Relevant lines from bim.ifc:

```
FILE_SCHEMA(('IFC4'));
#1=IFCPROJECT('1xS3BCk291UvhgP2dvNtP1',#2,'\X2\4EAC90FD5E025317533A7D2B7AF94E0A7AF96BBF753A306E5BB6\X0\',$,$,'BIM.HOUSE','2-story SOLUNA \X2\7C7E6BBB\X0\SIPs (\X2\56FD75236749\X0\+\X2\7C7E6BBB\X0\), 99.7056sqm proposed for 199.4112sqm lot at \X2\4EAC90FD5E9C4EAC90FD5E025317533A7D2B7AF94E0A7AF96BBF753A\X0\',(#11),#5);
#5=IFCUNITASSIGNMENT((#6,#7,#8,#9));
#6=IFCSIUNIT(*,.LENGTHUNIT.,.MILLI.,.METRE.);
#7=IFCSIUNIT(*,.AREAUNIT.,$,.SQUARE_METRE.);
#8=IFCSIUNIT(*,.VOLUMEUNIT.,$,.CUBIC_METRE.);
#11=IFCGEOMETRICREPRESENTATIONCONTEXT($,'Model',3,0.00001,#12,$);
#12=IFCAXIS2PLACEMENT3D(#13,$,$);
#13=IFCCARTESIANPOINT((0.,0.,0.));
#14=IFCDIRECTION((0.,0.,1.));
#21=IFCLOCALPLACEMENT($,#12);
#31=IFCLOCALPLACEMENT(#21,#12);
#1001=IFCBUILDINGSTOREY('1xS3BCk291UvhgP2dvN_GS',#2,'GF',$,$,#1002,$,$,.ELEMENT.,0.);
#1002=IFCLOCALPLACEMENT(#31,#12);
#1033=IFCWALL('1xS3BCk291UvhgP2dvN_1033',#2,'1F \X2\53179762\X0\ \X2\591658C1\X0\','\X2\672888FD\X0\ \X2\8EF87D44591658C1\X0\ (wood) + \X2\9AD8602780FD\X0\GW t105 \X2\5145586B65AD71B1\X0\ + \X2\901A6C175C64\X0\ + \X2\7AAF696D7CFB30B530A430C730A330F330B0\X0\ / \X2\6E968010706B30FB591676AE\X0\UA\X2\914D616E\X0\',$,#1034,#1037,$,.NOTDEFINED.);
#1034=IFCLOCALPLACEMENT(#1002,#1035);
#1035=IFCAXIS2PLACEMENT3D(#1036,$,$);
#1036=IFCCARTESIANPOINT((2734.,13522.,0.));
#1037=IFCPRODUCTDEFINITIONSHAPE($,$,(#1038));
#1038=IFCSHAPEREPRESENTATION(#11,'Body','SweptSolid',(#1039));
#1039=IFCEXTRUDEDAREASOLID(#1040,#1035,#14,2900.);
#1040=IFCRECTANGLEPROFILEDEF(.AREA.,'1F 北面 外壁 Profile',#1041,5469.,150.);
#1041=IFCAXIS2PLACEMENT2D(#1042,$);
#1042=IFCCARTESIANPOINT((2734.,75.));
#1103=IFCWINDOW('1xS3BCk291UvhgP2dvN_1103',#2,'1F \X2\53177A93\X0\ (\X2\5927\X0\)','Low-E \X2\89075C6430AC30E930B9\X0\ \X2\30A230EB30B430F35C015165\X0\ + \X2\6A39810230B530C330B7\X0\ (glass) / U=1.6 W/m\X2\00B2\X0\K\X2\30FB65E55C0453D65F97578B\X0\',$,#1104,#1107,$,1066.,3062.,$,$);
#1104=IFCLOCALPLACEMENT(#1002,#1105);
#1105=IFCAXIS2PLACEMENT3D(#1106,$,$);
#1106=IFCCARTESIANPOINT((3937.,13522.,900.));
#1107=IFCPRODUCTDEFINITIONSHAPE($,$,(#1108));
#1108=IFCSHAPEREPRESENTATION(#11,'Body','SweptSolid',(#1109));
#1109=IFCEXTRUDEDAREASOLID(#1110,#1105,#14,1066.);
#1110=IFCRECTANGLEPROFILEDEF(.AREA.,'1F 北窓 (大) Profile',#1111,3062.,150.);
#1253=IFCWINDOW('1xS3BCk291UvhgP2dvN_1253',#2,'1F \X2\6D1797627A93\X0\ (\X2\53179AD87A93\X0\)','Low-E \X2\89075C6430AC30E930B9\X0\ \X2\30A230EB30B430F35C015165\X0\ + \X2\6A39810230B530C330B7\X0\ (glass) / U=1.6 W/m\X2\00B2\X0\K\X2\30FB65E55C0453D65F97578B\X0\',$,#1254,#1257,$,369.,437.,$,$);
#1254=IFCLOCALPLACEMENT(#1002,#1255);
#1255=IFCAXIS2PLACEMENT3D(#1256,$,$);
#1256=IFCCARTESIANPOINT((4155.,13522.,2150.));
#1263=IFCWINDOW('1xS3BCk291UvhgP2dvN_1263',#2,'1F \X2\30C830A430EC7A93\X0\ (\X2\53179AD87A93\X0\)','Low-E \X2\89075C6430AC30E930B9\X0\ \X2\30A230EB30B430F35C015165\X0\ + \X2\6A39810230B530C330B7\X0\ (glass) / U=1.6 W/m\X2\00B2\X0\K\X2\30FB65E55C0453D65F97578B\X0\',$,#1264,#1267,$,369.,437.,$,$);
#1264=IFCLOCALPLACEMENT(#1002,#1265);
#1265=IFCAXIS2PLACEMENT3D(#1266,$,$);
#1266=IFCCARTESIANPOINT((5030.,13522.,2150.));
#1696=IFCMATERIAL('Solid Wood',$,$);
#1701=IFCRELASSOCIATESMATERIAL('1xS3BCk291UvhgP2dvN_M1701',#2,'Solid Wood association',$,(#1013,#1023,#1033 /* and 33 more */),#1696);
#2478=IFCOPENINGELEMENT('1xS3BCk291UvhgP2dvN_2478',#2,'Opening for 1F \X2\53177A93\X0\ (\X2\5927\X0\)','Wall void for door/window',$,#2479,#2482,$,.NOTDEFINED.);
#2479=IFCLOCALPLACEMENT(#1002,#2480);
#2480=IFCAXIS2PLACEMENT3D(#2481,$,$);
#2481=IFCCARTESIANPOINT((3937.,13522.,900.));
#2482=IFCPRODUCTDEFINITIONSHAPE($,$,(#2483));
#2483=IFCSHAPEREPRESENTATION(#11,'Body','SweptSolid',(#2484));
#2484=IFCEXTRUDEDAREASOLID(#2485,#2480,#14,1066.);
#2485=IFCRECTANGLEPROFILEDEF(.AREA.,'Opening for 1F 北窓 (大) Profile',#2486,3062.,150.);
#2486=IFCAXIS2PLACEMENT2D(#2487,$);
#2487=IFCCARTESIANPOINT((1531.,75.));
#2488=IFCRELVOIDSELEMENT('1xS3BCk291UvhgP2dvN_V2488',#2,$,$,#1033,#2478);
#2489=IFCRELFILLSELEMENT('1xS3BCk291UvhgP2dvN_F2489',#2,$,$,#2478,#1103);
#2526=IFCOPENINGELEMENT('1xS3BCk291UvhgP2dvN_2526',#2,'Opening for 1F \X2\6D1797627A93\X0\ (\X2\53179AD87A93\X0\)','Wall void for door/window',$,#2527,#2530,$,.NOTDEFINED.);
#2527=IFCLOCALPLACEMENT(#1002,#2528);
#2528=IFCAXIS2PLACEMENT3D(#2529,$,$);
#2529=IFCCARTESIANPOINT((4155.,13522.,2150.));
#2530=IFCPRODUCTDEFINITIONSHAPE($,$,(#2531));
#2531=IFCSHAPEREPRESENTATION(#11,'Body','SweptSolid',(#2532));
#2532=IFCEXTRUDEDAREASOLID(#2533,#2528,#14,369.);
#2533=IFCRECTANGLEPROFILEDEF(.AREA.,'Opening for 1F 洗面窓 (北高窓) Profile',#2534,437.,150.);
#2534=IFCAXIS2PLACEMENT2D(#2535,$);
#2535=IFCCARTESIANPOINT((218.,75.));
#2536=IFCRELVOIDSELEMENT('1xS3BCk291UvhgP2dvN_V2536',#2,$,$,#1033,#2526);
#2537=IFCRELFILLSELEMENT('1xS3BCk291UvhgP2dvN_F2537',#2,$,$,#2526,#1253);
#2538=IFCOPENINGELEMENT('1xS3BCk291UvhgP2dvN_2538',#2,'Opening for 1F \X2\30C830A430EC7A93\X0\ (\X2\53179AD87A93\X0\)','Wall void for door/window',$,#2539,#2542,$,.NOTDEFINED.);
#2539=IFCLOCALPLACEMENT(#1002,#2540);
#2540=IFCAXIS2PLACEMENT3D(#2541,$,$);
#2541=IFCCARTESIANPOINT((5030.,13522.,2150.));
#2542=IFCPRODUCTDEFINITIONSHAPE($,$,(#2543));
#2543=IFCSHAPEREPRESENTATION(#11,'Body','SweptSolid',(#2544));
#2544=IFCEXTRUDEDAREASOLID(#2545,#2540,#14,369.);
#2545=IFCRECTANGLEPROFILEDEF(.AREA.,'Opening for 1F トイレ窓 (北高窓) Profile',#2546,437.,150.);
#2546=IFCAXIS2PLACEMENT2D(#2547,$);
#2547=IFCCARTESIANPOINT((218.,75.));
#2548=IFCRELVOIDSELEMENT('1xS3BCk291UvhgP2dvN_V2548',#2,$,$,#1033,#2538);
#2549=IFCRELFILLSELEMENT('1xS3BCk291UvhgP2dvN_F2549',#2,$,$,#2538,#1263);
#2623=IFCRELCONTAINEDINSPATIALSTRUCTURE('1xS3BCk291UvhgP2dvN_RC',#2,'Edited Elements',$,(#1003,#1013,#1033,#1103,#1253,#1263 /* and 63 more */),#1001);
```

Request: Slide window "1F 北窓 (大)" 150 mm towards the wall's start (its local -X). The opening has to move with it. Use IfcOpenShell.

```python
import ifcopenshell
import ifcopenshell.api.geometry
import ifcopenshell.util.placement

model = ifcopenshell.open("bim.ifc")

window = model.by_guid("1xS3BCk291UvhgP2dvN_1103")
opening = window.FillsVoids[0].RelatingOpeningElement
wall = opening.VoidsElements[0].RelatingBuildingElement

wall_matrix = ifcopenshell.util.placement.get_local_placement(wall.ObjectPlacement)
shift = wall_matrix[:3, 0] * -150.0
before = ifcopenshell.util.placement.get_local_placement(window.ObjectPlacement)[:3, 3].copy()

# The window is not placed relative to its opening, so move both.
for product in (opening, window):
    matrix = ifcopenshell.util.placement.get_local_placement(product.ObjectPlacement)
    matrix[:3, 3] += shift
    ifcopenshell.api.geometry.edit_object_placement(model, product=product, matrix=matrix, is_si=False)

after = ifcopenshell.util.placement.get_local_placement(window.ObjectPlacement)[:3, 3]
print("window moved by", (after - before).round(3) + 0.0)

model.write("bim_rev.ifc")
```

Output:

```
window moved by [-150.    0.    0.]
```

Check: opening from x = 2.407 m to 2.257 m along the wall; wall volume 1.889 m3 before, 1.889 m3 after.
